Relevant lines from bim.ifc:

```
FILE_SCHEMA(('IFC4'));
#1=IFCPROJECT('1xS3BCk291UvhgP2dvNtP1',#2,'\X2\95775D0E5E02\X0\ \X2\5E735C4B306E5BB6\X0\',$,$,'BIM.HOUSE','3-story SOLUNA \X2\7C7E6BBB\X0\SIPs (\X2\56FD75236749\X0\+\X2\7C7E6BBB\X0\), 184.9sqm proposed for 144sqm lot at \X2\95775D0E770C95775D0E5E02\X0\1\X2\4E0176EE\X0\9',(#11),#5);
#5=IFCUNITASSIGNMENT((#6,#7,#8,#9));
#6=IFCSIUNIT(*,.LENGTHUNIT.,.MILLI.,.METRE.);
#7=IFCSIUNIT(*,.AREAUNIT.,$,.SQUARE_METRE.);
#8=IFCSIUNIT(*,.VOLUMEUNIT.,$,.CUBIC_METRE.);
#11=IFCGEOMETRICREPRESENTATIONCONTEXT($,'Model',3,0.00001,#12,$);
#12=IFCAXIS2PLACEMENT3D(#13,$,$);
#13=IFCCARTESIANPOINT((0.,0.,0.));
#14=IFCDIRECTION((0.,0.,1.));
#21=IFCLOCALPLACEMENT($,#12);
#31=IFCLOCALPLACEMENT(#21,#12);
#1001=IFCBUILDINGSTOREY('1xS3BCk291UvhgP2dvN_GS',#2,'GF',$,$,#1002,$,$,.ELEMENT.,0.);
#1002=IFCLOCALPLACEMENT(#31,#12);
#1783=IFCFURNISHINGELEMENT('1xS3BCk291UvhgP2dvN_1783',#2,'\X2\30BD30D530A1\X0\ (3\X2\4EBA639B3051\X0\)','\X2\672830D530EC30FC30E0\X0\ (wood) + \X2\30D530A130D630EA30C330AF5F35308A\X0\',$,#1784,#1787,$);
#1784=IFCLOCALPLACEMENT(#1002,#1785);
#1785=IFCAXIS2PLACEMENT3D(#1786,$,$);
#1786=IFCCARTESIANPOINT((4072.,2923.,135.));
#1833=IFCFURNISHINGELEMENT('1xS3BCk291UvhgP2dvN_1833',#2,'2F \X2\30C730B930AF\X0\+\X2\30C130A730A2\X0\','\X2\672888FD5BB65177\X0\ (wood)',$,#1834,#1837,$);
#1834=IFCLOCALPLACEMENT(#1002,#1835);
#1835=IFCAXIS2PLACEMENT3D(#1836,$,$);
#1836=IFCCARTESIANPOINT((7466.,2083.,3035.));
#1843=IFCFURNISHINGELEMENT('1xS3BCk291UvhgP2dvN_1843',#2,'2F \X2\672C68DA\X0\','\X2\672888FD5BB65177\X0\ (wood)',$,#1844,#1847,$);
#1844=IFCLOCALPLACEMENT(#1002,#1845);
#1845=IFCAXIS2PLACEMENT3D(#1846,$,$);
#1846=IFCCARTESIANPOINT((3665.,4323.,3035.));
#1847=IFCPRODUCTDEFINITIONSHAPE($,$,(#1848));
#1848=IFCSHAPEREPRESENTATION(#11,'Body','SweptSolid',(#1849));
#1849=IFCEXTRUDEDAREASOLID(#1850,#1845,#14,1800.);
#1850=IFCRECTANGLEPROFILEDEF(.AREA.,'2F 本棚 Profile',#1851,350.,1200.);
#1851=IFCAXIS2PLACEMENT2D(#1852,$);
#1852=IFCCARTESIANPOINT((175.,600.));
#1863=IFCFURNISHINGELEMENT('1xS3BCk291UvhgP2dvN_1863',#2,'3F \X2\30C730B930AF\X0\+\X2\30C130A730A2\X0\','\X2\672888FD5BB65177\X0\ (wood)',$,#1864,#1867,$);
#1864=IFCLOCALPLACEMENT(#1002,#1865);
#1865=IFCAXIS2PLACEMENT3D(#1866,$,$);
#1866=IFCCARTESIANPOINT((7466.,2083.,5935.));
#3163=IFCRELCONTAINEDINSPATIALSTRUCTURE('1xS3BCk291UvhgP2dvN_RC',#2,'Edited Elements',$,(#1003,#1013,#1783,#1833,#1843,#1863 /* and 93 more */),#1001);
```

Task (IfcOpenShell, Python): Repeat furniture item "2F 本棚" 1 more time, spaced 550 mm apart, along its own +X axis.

```python
import ifcopenshell
import ifcopenshell.api.geometry
import ifcopenshell.api.root
import ifcopenshell.util.element
import ifcopenshell.util.placement

model = ifcopenshell.open("bim.ifc")


def reuse_history(source, copy):
    """copy_class also copies each property set's owner history, people and application; keep the originals."""
    for rel in copy.IsDefinedBy:
        if rel.is_a("IfcRelDefinesByProperties") and (history := rel.RelatingPropertyDefinition.OwnerHistory):
            rel.RelatingPropertyDefinition.OwnerHistory = source.OwnerHistory
            ifcopenshell.util.element.remove_deep2(model, history)


source = model.by_guid("1xS3BCk291UvhgP2dvN_1843")
base = ifcopenshell.util.placement.get_local_placement(source.ObjectPlacement)
step = base[:3, 0] * 550.0

for i in range(1, 2):
    copy = ifcopenshell.api.root.copy_class(model, product=source)
    copy.Representation = ifcopenshell.util.element.copy_deep(
        model, source.Representation, exclude=["IfcGeometricRepresentationContext", "IfcRepresentationMap"]
    )
    reuse_history(source, copy)
    matrix = base.copy()
    matrix[:3, 3] += i * step
    print("added at", matrix[:3, 3].round(3) + 0.0)
    ifcopenshell.api.geometry.edit_object_placement(model, product=copy, matrix=matrix, is_si=False)

model.write("bim_v2.ifc")
```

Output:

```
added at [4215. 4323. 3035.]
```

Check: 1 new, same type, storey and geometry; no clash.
